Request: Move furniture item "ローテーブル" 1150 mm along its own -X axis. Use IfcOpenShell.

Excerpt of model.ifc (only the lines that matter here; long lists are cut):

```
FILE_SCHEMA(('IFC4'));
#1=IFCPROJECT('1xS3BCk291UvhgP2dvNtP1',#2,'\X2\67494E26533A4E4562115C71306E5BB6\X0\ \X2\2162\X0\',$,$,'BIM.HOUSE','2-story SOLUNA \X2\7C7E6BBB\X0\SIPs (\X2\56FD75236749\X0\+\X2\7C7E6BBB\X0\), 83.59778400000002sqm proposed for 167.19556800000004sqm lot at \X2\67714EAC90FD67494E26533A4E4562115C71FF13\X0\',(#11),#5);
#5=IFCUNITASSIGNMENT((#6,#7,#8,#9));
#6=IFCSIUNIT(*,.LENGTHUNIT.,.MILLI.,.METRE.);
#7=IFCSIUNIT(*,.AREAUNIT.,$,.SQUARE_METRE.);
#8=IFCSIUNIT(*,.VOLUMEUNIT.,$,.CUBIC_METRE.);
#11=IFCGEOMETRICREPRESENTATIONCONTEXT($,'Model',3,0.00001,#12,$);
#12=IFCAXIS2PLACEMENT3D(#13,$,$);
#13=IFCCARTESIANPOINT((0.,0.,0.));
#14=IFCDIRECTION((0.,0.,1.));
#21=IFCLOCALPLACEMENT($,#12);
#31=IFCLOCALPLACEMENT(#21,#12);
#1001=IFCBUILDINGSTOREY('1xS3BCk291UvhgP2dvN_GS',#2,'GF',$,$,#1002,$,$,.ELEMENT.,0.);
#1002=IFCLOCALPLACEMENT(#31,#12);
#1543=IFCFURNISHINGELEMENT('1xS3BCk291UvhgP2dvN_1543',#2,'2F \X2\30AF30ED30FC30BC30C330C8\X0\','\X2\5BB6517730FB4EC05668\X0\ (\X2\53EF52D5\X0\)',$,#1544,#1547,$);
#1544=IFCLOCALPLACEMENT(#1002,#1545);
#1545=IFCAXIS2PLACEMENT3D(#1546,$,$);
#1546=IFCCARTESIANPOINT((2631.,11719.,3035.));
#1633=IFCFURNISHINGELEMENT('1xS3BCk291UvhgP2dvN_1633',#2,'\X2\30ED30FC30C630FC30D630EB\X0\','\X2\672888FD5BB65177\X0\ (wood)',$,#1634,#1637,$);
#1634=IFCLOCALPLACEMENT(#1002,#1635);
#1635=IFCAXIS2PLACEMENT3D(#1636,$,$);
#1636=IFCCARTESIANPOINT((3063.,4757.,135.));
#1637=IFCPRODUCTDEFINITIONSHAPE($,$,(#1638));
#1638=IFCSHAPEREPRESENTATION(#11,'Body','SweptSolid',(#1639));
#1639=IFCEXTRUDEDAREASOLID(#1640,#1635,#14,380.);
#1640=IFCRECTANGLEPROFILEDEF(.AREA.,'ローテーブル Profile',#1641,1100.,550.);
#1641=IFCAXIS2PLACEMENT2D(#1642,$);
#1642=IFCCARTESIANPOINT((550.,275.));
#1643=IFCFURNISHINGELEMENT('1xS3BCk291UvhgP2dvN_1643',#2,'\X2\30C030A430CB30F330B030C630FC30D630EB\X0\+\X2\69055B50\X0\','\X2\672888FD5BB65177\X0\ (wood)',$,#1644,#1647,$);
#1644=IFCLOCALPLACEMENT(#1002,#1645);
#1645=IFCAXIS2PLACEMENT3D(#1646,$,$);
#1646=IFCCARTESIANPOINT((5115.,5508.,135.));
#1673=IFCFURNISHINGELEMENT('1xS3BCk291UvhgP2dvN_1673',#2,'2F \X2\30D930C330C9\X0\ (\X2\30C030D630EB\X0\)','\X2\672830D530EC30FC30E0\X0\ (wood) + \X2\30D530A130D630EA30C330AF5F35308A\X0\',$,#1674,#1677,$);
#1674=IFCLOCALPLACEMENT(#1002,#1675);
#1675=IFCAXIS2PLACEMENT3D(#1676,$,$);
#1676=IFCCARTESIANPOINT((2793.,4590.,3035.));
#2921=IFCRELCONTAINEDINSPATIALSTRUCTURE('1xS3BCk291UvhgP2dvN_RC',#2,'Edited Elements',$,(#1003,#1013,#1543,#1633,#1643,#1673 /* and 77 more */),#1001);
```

```python
import ifcopenshell
import ifcopenshell.api.geometry
import ifcopenshell.util.placement
import ifcopenshell.util.unit

model = ifcopenshell.open("model.ifc")
unit_scale = ifcopenshell.util.unit.calculate_unit_scale(model)

item = model.by_guid("1xS3BCk291UvhgP2dvN_1633")
matrix = ifcopenshell.util.placement.get_local_placement(item.ObjectPlacement)
matrix[:3, 3] -= matrix[:3, 0] * 1.15 / unit_scale
ifcopenshell.api.geometry.edit_object_placement(model, product=item, matrix=matrix, is_si=False)

print(ifcopenshell.util.placement.get_local_placement(item.ObjectPlacement).round(3) + 0.0)

model.write("model_v2.ifc")
```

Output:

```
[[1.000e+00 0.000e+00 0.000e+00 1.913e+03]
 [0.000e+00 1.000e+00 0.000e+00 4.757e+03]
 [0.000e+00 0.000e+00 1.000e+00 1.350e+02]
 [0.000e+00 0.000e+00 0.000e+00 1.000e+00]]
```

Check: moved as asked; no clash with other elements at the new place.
